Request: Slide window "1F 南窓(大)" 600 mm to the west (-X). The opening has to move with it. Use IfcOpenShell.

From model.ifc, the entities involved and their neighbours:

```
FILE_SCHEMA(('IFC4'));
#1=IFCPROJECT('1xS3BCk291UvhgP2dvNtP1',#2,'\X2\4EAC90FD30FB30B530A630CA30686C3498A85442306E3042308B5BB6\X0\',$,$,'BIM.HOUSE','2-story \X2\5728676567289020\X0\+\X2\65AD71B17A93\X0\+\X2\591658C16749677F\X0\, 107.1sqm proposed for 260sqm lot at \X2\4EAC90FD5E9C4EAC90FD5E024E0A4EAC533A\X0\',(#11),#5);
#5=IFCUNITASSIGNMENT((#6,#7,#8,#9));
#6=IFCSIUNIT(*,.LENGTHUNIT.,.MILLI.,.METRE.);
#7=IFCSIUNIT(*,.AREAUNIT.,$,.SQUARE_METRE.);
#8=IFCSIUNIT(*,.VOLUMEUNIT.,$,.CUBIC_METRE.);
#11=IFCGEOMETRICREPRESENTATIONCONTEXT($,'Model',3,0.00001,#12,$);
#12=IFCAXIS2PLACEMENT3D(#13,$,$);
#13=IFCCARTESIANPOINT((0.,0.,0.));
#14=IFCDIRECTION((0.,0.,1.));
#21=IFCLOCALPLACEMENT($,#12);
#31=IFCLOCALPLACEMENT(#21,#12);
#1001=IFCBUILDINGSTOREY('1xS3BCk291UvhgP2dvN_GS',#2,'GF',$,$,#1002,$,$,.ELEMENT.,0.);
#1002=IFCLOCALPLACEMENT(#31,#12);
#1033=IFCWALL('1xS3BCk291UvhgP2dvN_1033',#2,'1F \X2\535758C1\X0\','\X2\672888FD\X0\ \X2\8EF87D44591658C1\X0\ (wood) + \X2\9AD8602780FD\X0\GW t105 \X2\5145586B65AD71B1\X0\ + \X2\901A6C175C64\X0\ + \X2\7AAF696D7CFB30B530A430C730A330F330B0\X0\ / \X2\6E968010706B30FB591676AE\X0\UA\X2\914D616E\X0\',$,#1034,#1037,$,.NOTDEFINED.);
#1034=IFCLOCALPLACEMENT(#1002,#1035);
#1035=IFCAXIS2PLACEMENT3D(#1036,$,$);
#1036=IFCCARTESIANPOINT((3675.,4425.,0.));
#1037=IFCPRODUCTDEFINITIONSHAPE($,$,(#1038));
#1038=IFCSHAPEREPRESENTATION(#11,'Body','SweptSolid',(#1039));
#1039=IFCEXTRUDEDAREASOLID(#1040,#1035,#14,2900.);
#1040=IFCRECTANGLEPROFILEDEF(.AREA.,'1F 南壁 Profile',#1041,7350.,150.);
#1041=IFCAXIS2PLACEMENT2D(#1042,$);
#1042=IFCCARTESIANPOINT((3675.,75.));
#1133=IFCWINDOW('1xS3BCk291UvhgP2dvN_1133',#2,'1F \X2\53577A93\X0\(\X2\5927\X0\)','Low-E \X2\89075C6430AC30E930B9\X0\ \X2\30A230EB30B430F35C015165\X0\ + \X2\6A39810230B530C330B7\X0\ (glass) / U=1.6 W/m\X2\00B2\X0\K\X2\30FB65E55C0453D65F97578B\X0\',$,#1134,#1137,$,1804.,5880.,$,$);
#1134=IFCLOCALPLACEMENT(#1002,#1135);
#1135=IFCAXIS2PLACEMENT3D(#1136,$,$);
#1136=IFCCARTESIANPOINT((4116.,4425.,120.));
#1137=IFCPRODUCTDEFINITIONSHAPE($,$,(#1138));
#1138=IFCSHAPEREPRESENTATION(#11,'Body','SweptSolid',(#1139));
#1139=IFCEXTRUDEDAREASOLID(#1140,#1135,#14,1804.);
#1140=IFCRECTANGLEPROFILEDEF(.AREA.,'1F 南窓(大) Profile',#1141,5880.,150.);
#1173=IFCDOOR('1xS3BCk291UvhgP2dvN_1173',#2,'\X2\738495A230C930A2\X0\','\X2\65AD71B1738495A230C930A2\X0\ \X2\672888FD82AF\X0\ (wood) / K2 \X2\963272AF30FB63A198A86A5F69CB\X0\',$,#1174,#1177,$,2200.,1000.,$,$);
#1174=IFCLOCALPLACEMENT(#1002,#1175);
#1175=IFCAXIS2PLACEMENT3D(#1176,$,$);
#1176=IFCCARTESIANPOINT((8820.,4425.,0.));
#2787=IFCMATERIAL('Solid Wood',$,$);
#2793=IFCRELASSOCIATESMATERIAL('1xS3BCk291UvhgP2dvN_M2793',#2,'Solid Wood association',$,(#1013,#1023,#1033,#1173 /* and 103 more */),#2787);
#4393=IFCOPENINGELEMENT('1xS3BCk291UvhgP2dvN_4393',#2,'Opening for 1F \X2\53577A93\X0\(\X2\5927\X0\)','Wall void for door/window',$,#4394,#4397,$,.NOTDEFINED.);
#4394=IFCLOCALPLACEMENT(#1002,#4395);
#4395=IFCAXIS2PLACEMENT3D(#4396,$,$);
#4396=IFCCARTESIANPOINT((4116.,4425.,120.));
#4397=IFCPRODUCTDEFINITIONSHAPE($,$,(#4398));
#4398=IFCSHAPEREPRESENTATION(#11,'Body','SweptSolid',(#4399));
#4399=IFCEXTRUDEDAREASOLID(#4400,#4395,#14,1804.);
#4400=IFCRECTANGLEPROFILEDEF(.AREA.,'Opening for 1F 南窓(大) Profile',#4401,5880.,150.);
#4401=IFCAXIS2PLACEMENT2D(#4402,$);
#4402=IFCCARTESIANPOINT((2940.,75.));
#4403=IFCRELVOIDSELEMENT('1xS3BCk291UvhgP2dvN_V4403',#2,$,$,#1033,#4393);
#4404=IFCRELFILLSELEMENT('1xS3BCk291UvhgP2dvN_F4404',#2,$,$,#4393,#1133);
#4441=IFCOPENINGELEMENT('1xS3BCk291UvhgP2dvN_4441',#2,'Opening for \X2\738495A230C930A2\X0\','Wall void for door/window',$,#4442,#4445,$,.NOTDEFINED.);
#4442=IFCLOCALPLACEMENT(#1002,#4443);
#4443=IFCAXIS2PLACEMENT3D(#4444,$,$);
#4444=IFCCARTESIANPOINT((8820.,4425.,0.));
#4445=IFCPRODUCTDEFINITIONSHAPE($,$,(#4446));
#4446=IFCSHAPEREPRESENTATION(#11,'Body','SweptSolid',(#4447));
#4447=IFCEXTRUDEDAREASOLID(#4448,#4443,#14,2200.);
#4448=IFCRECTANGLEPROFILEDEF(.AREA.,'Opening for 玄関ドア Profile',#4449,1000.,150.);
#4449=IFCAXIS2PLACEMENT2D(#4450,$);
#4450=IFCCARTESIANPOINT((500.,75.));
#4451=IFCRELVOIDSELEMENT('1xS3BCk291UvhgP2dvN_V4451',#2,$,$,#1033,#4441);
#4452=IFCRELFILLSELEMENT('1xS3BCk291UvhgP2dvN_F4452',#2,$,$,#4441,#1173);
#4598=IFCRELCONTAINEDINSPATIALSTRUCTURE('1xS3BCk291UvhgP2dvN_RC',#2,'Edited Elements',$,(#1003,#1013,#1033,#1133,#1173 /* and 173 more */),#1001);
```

```python
import ifcopenshell
import ifcopenshell.api.geometry
import ifcopenshell.util.placement

model = ifcopenshell.open("model.ifc")

window = model.by_guid("1xS3BCk291UvhgP2dvN_1133")
opening = window.FillsVoids[0].RelatingOpeningElement
wall = opening.VoidsElements[0].RelatingBuildingElement

wall_matrix = ifcopenshell.util.placement.get_local_placement(wall.ObjectPlacement)
shift = wall_matrix[:3, 0] * -600.0
before = ifcopenshell.util.placement.get_local_placement(window.ObjectPlacement)[:3, 3].copy()

# The window is not placed relative to its opening, so move both.
for product in (opening, window):
    matrix = ifcopenshell.util.placement.get_local_placement(product.ObjectPlacement)
    matrix[:3, 3] += shift
    ifcopenshell.api.geometry.edit_object_placement(model, product=product, matrix=matrix, is_si=False)

after = ifcopenshell.util.placement.get_local_placement(window.ObjectPlacement)[:3, 3]
print("window moved by", (after - before).round(3) + 0.0)

model.write("model_v2.ifc")
```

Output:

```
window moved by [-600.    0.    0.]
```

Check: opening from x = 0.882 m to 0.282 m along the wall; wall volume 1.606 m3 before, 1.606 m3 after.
